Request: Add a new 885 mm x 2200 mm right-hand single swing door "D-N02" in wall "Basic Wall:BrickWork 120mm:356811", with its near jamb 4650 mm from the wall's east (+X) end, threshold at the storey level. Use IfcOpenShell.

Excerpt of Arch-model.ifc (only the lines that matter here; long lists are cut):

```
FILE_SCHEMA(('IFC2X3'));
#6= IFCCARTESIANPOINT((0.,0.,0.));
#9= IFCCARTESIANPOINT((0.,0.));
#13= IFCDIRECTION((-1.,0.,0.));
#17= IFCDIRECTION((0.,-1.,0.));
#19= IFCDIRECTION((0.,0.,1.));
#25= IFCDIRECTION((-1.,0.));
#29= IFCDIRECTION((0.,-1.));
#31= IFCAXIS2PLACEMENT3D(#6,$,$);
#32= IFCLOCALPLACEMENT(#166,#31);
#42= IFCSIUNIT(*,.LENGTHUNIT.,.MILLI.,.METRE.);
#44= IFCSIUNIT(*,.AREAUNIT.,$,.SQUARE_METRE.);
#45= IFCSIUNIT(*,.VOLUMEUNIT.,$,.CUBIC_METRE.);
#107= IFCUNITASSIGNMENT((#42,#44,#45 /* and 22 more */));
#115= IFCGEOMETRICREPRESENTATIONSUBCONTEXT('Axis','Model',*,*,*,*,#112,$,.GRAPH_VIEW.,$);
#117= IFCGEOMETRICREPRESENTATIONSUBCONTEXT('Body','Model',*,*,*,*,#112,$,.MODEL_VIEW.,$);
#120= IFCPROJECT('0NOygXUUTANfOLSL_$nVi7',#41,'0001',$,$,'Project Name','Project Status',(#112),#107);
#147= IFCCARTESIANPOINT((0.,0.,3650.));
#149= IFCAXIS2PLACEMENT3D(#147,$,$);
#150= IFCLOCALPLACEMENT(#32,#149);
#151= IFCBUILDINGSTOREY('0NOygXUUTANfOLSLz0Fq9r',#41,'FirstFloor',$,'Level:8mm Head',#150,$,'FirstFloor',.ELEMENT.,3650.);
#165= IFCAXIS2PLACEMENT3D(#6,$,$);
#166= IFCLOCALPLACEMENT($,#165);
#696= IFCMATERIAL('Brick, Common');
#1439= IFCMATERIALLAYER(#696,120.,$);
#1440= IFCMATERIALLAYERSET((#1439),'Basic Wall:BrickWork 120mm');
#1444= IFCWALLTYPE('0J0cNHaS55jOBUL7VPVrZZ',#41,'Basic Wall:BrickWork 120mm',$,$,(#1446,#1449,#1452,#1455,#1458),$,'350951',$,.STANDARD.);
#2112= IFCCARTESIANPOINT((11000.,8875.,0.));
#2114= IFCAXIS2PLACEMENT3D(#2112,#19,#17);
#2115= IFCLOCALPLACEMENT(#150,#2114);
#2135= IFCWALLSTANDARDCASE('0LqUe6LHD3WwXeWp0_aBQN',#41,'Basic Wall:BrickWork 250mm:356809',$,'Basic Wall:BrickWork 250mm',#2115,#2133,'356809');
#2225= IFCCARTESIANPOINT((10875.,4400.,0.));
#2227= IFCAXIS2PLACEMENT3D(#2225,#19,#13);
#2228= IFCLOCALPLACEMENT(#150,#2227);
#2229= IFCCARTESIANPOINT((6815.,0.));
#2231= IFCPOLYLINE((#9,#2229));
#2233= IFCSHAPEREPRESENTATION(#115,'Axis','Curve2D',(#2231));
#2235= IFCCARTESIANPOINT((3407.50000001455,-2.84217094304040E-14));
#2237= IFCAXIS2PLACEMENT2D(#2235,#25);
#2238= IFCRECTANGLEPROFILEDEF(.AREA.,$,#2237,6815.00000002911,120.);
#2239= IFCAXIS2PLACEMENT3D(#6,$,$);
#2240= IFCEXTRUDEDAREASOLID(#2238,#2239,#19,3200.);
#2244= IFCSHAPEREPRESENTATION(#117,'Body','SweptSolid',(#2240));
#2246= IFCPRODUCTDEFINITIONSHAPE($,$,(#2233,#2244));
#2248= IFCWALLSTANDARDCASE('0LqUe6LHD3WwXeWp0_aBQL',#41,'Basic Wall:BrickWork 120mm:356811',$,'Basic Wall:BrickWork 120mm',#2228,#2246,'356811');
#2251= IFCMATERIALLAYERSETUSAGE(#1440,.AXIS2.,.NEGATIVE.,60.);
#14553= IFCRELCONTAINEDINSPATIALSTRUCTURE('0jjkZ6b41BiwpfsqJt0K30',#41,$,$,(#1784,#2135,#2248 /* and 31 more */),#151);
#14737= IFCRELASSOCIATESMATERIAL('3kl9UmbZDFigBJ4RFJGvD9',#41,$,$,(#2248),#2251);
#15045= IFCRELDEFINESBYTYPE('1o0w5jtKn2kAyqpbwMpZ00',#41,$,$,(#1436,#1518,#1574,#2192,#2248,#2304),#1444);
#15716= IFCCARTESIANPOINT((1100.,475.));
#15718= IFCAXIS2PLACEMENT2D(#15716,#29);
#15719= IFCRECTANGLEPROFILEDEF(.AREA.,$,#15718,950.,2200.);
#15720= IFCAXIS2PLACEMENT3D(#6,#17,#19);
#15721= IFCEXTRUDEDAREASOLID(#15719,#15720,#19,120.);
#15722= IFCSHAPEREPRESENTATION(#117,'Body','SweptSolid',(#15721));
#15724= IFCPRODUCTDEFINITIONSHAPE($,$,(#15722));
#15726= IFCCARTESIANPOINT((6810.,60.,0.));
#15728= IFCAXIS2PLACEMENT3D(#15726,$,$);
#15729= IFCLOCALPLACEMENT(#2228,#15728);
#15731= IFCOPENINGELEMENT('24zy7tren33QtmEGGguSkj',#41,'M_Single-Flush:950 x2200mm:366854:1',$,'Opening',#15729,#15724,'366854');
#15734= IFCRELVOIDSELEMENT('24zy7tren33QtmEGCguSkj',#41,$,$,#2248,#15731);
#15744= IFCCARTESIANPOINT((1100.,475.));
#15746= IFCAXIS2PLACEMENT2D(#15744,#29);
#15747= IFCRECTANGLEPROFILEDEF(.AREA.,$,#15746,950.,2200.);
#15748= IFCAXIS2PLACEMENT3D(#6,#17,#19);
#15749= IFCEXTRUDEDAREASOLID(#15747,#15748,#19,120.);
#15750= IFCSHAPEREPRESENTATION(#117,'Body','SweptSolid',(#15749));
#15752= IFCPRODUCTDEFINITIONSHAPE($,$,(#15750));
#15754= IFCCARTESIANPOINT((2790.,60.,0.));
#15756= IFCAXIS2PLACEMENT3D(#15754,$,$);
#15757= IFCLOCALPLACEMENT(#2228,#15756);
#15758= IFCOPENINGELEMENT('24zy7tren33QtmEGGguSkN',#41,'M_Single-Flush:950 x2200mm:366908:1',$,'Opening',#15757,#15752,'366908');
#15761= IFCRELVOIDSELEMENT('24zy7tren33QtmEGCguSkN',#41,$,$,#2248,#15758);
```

```python
import numpy as np
import ifcopenshell
import ifcopenshell.api.feature
import ifcopenshell.api.geometry
import ifcopenshell.api.root
import ifcopenshell.api.spatial
import ifcopenshell.api.type
import ifcopenshell.geom
import ifcopenshell.util.element
import ifcopenshell.util.placement
import ifcopenshell.util.representation
import ifcopenshell.util.shape
import ifcopenshell.util.unit

model = ifcopenshell.open("Arch-model.ifc")
unit_scale = ifcopenshell.util.unit.calculate_unit_scale(model)
settings = ifcopenshell.geom.settings()


def volume(element):
    """Net volume in cubic metres, openings subtracted."""
    shape = ifcopenshell.geom.create_shape(settings, element)
    return ifcopenshell.util.shape.get_volume(shape.geometry)


wall = model.by_guid("0LqUe6LHD3WwXeWp0_aBQL")
storey = ifcopenshell.util.element.get_container(wall, ifc_class="IfcBuildingStorey")
context = ifcopenshell.util.representation.get_context(model, "Model", "Body", "MODEL_VIEW")
before = volume(wall)

width, height, from_end, sill = 0.885, 2.2, 4.65, 0.0  # metres

# The wall runs along its own X axis, and the end named is its -X end.
wall_shape = ifcopenshell.geom.create_shape(settings, wall)
x, y, z = ifcopenshell.util.shape.get_vertices(wall_shape.geometry).T
start = x.min() + from_end
face, thickness = float(y.min()), float(y.max() - y.min())
wall_matrix = ifcopenshell.util.placement.get_local_placement(wall.ObjectPlacement)
level = ifcopenshell.util.placement.get_local_placement(storey.ObjectPlacement)[2, 3]


def in_wall(x, y):
    """Placement at x, y metres in the wall's axes, at sill height."""
    matrix = wall_matrix.copy()
    matrix[:, 3] = wall_matrix @ np.array([x / unit_scale, y / unit_scale, 0.0, 1.0])
    matrix[2, 3] = level + sill / unit_scale
    return matrix


# Opening: a box that overshoots both wall faces by 50 mm.
opening = ifcopenshell.api.root.create_entity(model, ifc_class="IfcOpeningElement")
box = ifcopenshell.api.geometry.add_wall_representation(
    model, context=context, length=width, height=height, thickness=thickness + 0.1
)
ifcopenshell.api.geometry.assign_representation(model, product=opening, representation=box)
ifcopenshell.api.geometry.edit_object_placement(model, product=opening, matrix=in_wall(start, face - 0.05), is_si=False)
ifcopenshell.api.feature.add_feature(model, feature=opening, element=wall)

door = ifcopenshell.api.root.create_entity(model, ifc_class="IfcDoor", name="D-N02")
door.OverallWidth, door.OverallHeight = width / unit_scale, height / unit_scale
body = ifcopenshell.api.geometry.add_door_representation(
    model,
    context=context,
    overall_width=door.OverallWidth,
    overall_height=door.OverallHeight,
    operation_type="SINGLE_SWING_RIGHT",
    lining_properties={"LiningDepth": thickness / unit_scale, "ThresholdDepth": thickness / unit_scale},
)
ifcopenshell.api.geometry.assign_representation(model, product=door, representation=body)
ifcopenshell.api.spatial.assign_container(model, products=[door], relating_structure=storey)
fills = ifcopenshell.api.feature.add_filling(model, opening=opening, element=door)
fills.OwnerHistory = door.OwnerHistory  # required in IFC2X3

# IFC2X3 keeps the operation on the door style.
style = ifcopenshell.api.root.create_entity(model, ifc_class="IfcDoorStyle", name="D-N02")
style.OperationType, style.ConstructionType = "SINGLE_SWING_RIGHT", "NOTDEFINED"
style.ParameterTakesPrecedence = style.Sizeable = False
ifcopenshell.api.type.assign_type(model, related_objects=[door], relating_type=style)

# The lining spans the wall, so the door starts at the wall face.
ifcopenshell.api.geometry.edit_object_placement(model, product=door, matrix=in_wall(start, face), is_si=False)

after = volume(wall)

print(f"wall volume {before:.3f} -> {after:.3f} m3")

model.write("Arch-model_edited.ifc")
```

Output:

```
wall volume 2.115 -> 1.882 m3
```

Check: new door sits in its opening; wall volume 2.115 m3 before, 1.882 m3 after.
